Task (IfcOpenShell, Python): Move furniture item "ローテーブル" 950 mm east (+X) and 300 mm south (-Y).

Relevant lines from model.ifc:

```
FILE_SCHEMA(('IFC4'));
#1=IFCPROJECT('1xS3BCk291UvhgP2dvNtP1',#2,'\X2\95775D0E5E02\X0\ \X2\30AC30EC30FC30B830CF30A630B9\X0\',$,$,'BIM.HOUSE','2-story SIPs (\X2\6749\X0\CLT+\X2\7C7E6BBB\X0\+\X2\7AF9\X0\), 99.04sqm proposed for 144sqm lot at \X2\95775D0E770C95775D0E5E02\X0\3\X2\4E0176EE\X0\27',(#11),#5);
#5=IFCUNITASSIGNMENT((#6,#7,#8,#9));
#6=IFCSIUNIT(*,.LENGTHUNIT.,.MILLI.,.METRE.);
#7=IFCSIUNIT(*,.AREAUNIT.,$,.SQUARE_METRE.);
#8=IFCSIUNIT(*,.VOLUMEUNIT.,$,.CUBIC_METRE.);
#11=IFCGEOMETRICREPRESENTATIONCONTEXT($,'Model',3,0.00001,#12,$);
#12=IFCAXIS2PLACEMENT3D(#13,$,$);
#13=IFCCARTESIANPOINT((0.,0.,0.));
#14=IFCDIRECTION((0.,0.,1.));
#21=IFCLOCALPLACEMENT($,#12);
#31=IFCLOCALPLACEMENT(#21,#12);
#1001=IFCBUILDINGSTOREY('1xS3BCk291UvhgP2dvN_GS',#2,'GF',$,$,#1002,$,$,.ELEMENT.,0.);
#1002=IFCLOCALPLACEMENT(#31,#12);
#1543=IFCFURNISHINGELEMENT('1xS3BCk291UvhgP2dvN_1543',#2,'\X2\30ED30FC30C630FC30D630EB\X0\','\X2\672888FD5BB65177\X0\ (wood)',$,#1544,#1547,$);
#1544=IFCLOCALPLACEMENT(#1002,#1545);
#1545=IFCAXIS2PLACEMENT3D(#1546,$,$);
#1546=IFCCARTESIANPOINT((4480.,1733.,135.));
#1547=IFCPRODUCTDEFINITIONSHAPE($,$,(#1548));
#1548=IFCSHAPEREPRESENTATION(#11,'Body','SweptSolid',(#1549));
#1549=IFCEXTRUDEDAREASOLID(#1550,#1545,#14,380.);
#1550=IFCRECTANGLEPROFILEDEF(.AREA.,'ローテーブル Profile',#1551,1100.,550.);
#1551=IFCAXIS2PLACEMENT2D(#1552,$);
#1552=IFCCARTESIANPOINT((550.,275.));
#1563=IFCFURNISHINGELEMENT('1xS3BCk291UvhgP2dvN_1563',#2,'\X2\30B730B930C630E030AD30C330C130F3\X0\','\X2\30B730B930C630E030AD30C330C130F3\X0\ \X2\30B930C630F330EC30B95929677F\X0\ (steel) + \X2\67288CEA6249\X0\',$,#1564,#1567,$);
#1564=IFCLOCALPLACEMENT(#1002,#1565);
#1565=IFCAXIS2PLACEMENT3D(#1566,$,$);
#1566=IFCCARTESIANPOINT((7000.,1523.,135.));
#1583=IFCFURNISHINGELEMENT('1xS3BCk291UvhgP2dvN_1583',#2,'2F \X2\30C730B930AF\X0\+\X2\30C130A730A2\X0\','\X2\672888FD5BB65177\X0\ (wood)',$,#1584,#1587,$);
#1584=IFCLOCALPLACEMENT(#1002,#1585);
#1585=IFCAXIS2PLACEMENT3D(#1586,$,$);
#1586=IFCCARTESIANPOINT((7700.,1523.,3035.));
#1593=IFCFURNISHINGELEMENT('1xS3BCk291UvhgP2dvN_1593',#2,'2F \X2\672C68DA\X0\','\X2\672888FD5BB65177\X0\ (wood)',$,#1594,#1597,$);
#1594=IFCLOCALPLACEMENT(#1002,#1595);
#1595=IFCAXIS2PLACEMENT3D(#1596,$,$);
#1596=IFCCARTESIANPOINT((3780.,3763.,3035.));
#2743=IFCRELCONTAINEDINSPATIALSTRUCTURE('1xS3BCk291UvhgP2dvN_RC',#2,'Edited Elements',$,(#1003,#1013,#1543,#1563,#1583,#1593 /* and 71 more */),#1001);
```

```python
import ifcopenshell
import ifcopenshell.api.geometry
import ifcopenshell.util.placement

model = ifcopenshell.open("model.ifc")

item = model.by_guid("1xS3BCk291UvhgP2dvN_1543")
matrix = ifcopenshell.util.placement.get_local_placement(item.ObjectPlacement)
matrix[0, 3] += 950.0
matrix[1, 3] -= 300.0
ifcopenshell.api.geometry.edit_object_placement(model, product=item, matrix=matrix, is_si=False)

print(ifcopenshell.util.placement.get_local_placement(item.ObjectPlacement).round(3) + 0.0)

model.write("model_rev.ifc")
```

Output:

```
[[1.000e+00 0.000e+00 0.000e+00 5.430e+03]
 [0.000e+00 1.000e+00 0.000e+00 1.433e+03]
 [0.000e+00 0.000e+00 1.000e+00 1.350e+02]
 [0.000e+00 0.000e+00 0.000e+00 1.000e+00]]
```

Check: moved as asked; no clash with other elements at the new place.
